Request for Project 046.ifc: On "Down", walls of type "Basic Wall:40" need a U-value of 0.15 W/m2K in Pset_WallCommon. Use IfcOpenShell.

First a look at what the model holds.

```python
import ifcopenshell
import ifcopenshell.util.element

model = ifcopenshell.open("Project 046.ifc")
print(model.schema)
storey = next(s for s in model.by_type("IfcBuildingStorey") if s.Name == "Down")
walls = [e for e in ifcopenshell.util.element.get_decomposition(storey) if e.is_a("IfcWall")]
seen = {}
for e in walls:
    element_type = ifcopenshell.util.element.get_type(e)
    key = (element_type.Name if element_type != e and element_type else None, ifcopenshell.util.element.get_pset(e, "Pset_WallCommon", "ThermalTransmittance"))
    seen[key] = seen.get(key, 0) + 1
for (name, value), count in sorted(seen.items(), key=str):
    print(count, "x", name, "|", value)
```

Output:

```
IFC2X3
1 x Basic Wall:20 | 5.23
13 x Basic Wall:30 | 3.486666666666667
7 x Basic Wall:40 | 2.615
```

```python
import ifcopenshell
import ifcopenshell.api.pset
import ifcopenshell.util.element

model = ifcopenshell.open("Project 046.ifc")

storey = next(s for s in model.by_type("IfcBuildingStorey") if s.Name == "Down")
walls = [e for e in ifcopenshell.util.element.get_decomposition(storey) if e.is_a("IfcWall")]

count = 0
for e in walls:
    element_type = ifcopenshell.util.element.get_type(e)
    if element_type in (None, e) or element_type.Name != "Basic Wall:40":
        continue
    # add_pset returns the element's existing set when there is one.
    pset = ifcopenshell.api.pset.add_pset(model, product=e, name="Pset_WallCommon")
    ifcopenshell.api.pset.edit_pset(model, pset=pset, properties={"ThermalTransmittance": 0.15})
    count += 1

print(count, "walls updated")

model.write("Project 046_rev.ifc")
```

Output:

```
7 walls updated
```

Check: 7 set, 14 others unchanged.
